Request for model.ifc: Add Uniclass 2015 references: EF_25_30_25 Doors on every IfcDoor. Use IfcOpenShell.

First a look at what the model holds.

```python
import ifcopenshell

model = ifcopenshell.open("model.ifc")
print(model.schema)
print("classifications:", [c.Name for c in model.by_type("IfcClassification")])
for ifc_class in ("IfcDoor", "IfcRoof", "IfcStair", "IfcWall", "IfcWindow"):
    print(ifc_class, len(model.by_type(ifc_class)))
```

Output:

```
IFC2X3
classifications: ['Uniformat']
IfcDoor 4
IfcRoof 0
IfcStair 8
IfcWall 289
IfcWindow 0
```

```python
import ifcopenshell
import ifcopenshell.api.classification

model = ifcopenshell.open("model.ifc")

# IFC2X3 requires Source and Edition and has no link from the project to the system.
system = model.create_entity("IfcClassification", Source="NBS", Edition="2015", Name="Uniclass 2015")

codes = {
    "IfcDoor": ("EF_25_30_25", "Doors"),
}
for ifc_class, (code, name) in codes.items():
    products = model.by_type(ifc_class)
    ifcopenshell.api.classification.add_reference(
        model, products=products, classification=system, identification=code, name=name
    )
    print(code, len(products))

model.write("model_updated.ifc")
```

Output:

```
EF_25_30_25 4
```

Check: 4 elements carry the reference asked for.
